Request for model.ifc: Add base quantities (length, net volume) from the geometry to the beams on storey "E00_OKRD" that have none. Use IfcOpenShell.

First a look at what the model holds.

```python
import ifcopenshell
import ifcopenshell.util.element
import ifcopenshell.util.unit

model = ifcopenshell.open("model.ifc")
print(model.schema)
for unit_type in ("LENGTHUNIT", "AREAUNIT", "VOLUMEUNIT"):
    print(unit_type, ifcopenshell.util.unit.calculate_unit_scale(model, unit_type))
storey = next(s for s in model.by_type("IfcBuildingStorey") if s.Name == "E00_OKRD")
beams = [e for e in ifcopenshell.util.element.get_decomposition(storey) if e.is_a("IfcBeam")]
for e in sorted(beams, key=lambda e: e.id()):
    print(e.id(), e.is_a(), e.Name, list(ifcopenshell.util.element.get_psets(e, qtos_only=True)), sep=" | ")
```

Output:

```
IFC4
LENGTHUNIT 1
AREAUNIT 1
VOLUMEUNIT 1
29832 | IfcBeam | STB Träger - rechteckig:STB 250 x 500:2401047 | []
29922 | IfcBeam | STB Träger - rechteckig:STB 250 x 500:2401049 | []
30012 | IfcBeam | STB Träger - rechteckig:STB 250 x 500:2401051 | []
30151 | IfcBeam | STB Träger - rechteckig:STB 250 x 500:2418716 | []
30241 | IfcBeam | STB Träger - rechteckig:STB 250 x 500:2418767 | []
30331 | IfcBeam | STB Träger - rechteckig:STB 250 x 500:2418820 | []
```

```python
import ifcopenshell
import ifcopenshell.api.pset
import ifcopenshell.geom
import ifcopenshell.util.element
import ifcopenshell.util.shape
import ifcopenshell.util.unit

model = ifcopenshell.open("model.ifc")
unit_scale = ifcopenshell.util.unit.calculate_unit_scale(model)
volume_scale = ifcopenshell.util.unit.calculate_unit_scale(model, "VOLUMEUNIT")
settings = ifcopenshell.geom.settings()

storey = next(s for s in model.by_type("IfcBuildingStorey") if s.Name == "E00_OKRD")
beams = [e for e in ifcopenshell.util.element.get_decomposition(storey) if e.is_a("IfcBeam")]

for e in sorted(beams, key=lambda e: e.id()):
    if ifcopenshell.util.element.get_psets(e, qtos_only=True, should_inherit=False):
        continue
    # Geometry comes back in metres, in the element's own axes.
    shape = ifcopenshell.geom.create_shape(settings, e)
    values = {
        "Length": ifcopenshell.util.shape.get_max_xyz(shape.geometry) / unit_scale,
        "NetVolume": ifcopenshell.util.shape.get_volume(shape.geometry) / volume_scale,
    }
    qto = ifcopenshell.api.pset.add_qto(model, product=e, name="Qto_BeamBaseQuantities")
    ifcopenshell.api.pset.edit_qto(model, qto=qto, properties=values)
    print(e.id(), {k: round(v, 3) for k, v in values.items()})

model.write("model_v2.ifc")
```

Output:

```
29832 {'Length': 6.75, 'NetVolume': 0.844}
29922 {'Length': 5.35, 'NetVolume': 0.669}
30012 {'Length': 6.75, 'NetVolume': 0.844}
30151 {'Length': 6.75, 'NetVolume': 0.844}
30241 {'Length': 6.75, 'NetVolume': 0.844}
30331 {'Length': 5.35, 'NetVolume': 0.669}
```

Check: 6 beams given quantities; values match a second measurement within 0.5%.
